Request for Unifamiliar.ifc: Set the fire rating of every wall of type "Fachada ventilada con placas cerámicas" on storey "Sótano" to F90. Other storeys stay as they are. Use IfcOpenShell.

First a look at what the model holds.

```python
import ifcopenshell
import ifcopenshell.util.element

model = ifcopenshell.open("Unifamiliar.ifc")
print(model.schema)
storey = next(s for s in model.by_type("IfcBuildingStorey") if s.Name == "Sótano")
walls = [e for e in ifcopenshell.util.element.get_decomposition(storey) if e.is_a("IfcWall")]
seen = {}
for e in walls:
    element_type = ifcopenshell.util.element.get_type(e)
    key = (element_type.Name if element_type != e and element_type else None, ifcopenshell.util.element.get_pset(e, "Pset_WallCommon", "FireRating"))
    seen[key] = seen.get(key, 0) + 1
for (name, value), count in sorted(seen.items(), key=str):
    print(count, "x", name, "|", value)
```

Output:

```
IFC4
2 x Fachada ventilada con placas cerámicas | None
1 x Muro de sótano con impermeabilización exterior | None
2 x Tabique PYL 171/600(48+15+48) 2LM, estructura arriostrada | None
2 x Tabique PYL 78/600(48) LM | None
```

```python
import ifcopenshell
import ifcopenshell.api.pset
import ifcopenshell.util.element

model = ifcopenshell.open("Unifamiliar.ifc")

storey = next(s for s in model.by_type("IfcBuildingStorey") if s.Name == "Sótano")
walls = [e for e in ifcopenshell.util.element.get_decomposition(storey) if e.is_a("IfcWall")]

count = 0
for e in walls:
    element_type = ifcopenshell.util.element.get_type(e)
    if element_type in (None, e) or element_type.Name != "Fachada ventilada con placas cerámicas":
        continue
    # add_pset returns the element's existing set when there is one.
    pset = ifcopenshell.api.pset.add_pset(model, product=e, name="Pset_WallCommon")
    ifcopenshell.api.pset.edit_pset(model, pset=pset, properties={"FireRating": "F90"})
    count += 1

print(count, "walls updated")

model.write("Unifamiliar_rev.ifc")
```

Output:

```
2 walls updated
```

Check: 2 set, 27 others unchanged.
